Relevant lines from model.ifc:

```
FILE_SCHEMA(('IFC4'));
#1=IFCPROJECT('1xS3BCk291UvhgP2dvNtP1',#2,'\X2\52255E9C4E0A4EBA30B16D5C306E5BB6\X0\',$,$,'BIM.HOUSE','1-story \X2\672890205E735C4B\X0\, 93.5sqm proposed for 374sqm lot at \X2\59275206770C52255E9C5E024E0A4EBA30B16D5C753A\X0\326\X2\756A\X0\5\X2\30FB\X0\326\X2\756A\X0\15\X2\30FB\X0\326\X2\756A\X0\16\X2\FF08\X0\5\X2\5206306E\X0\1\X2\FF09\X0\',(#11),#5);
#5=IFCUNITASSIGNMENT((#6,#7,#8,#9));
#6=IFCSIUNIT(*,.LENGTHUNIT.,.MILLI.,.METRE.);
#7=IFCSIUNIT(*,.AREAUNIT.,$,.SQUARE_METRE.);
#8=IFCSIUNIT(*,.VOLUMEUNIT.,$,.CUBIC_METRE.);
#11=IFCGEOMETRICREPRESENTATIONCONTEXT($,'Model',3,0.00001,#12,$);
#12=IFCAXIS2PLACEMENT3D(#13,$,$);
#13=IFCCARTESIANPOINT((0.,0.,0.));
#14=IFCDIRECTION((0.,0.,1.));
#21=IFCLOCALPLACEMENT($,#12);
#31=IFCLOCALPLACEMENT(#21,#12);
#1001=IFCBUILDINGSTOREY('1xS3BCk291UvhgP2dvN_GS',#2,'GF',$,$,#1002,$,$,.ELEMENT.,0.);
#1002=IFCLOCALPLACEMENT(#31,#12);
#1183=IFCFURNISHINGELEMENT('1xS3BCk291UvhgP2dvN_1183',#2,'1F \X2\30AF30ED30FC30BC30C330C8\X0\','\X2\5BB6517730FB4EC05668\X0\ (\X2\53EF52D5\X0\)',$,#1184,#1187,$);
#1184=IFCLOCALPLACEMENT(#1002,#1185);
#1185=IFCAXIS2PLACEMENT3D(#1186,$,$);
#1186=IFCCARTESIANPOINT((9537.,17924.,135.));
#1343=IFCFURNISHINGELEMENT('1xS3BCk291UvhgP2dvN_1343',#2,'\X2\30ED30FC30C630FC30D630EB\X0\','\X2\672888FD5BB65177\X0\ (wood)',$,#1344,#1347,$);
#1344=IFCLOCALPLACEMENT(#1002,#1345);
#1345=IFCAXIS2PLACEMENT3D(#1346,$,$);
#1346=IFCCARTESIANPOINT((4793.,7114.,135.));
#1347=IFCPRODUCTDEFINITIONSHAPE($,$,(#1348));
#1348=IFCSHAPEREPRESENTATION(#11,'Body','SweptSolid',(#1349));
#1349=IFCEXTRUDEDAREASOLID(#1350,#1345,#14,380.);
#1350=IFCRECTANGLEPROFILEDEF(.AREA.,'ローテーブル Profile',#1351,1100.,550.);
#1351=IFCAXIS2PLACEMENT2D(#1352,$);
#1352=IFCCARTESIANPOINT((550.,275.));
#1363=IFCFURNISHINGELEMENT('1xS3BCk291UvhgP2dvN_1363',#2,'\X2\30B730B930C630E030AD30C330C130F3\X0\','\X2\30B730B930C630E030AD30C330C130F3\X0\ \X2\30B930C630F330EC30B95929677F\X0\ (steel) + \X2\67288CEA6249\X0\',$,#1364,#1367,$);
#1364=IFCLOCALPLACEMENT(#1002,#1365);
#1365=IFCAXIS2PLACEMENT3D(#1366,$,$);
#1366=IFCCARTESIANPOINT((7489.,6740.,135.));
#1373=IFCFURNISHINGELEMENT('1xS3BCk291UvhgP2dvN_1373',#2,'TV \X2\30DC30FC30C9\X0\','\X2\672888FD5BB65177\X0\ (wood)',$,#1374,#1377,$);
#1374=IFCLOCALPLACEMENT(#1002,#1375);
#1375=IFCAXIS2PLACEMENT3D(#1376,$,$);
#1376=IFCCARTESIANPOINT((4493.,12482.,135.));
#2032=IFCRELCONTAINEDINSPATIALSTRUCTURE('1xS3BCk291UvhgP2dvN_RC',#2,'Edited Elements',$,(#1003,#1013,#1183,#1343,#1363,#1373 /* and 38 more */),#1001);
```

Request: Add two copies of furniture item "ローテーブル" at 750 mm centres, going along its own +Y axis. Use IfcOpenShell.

```python
import ifcopenshell
import ifcopenshell.api.geometry
import ifcopenshell.api.root
import ifcopenshell.util.element
import ifcopenshell.util.placement
import ifcopenshell.util.unit

model = ifcopenshell.open("model.ifc")
unit_scale = ifcopenshell.util.unit.calculate_unit_scale(model)


def reuse_history(source, copy):
    """copy_class also copies each property set's owner history, people and application; keep the originals."""
    for rel in copy.IsDefinedBy:
        if rel.is_a("IfcRelDefinesByProperties") and (history := rel.RelatingPropertyDefinition.OwnerHistory):
            rel.RelatingPropertyDefinition.OwnerHistory = source.OwnerHistory
            ifcopenshell.util.element.remove_deep2(model, history)


source = model.by_guid("1xS3BCk291UvhgP2dvN_1343")
base = ifcopenshell.util.placement.get_local_placement(source.ObjectPlacement)
step = base[:3, 1] * 0.75 / unit_scale

for i in range(1, 3):
    copy = ifcopenshell.api.root.copy_class(model, product=source)
    copy.Representation = ifcopenshell.util.element.copy_deep(
        model, source.Representation, exclude=["IfcGeometricRepresentationContext", "IfcRepresentationMap"]
    )
    reuse_history(source, copy)
    matrix = base.copy()
    matrix[:3, 3] += i * step
    print("added at", matrix[:3, 3].round(3) + 0.0)
    ifcopenshell.api.geometry.edit_object_placement(model, product=copy, matrix=matrix, is_si=False)

model.write("model_v2.ifc")
```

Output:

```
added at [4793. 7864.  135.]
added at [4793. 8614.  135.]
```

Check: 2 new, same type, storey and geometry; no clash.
